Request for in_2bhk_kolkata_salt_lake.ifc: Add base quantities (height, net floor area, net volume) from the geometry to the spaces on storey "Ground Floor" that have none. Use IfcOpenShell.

First a look at what the model holds.

```python
import ifcopenshell
import ifcopenshell.util.element
import ifcopenshell.util.unit

model = ifcopenshell.open("in_2bhk_kolkata_salt_lake.ifc")
print(model.schema)
for unit_type in ("LENGTHUNIT", "AREAUNIT", "VOLUMEUNIT"):
    print(unit_type, ifcopenshell.util.unit.calculate_unit_scale(model, unit_type))
storey = next(s for s in model.by_type("IfcBuildingStorey") if s.Name == "Ground Floor")
spaces = [e for e in ifcopenshell.util.element.get_decomposition(storey) if e.is_a("IfcSpace")]
for e in sorted(spaces, key=lambda e: e.id()):
    print(e.id(), e.is_a(), e.Name, list(ifcopenshell.util.element.get_psets(e, qtos_only=True)), sep=" | ")
```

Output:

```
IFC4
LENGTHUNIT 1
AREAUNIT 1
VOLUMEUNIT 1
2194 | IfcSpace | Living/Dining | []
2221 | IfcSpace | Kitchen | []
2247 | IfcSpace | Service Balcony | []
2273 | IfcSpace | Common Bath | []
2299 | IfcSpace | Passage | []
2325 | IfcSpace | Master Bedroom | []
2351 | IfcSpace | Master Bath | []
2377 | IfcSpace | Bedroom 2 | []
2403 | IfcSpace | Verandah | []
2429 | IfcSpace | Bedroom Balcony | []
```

```python
import ifcopenshell
import ifcopenshell.api.pset
import ifcopenshell.geom
import ifcopenshell.util.element
import ifcopenshell.util.shape
import ifcopenshell.util.unit

model = ifcopenshell.open("in_2bhk_kolkata_salt_lake.ifc")
unit_scale = ifcopenshell.util.unit.calculate_unit_scale(model)
area_scale = ifcopenshell.util.unit.calculate_unit_scale(model, "AREAUNIT")
volume_scale = ifcopenshell.util.unit.calculate_unit_scale(model, "VOLUMEUNIT")
settings = ifcopenshell.geom.settings()

storey = next(s for s in model.by_type("IfcBuildingStorey") if s.Name == "Ground Floor")
spaces = [e for e in ifcopenshell.util.element.get_decomposition(storey) if e.is_a("IfcSpace")]

for e in sorted(spaces, key=lambda e: e.id()):
    if ifcopenshell.util.element.get_psets(e, qtos_only=True, should_inherit=False):
        continue
    # Geometry comes back in metres, in the element's own axes.
    shape = ifcopenshell.geom.create_shape(settings, e)
    values = {
        "Height": ifcopenshell.util.shape.get_z(shape.geometry) / unit_scale,
        "NetFloorArea": ifcopenshell.util.shape.get_footprint_area(shape.geometry) / area_scale,
        "NetVolume": ifcopenshell.util.shape.get_volume(shape.geometry) / volume_scale,
    }
    qto = ifcopenshell.api.pset.add_qto(model, product=e, name="Qto_SpaceBaseQuantities")
    ifcopenshell.api.pset.edit_qto(model, qto=qto, properties=values)
    print(e.id(), {k: round(v, 3) for k, v in values.items()})

model.write("in_2bhk_kolkata_salt_lake_rev.ifc")
```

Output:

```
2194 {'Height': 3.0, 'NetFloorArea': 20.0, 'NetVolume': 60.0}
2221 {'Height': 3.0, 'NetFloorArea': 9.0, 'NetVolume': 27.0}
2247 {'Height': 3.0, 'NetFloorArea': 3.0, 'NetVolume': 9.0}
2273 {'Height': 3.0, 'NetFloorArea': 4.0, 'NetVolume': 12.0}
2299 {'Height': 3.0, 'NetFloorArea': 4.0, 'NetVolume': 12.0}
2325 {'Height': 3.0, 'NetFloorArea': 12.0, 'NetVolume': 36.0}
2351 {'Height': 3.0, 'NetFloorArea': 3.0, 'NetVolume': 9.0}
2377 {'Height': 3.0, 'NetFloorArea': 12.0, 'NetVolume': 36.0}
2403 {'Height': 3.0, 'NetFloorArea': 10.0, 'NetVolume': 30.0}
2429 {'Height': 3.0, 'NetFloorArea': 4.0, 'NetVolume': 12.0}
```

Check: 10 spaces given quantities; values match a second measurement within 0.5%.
